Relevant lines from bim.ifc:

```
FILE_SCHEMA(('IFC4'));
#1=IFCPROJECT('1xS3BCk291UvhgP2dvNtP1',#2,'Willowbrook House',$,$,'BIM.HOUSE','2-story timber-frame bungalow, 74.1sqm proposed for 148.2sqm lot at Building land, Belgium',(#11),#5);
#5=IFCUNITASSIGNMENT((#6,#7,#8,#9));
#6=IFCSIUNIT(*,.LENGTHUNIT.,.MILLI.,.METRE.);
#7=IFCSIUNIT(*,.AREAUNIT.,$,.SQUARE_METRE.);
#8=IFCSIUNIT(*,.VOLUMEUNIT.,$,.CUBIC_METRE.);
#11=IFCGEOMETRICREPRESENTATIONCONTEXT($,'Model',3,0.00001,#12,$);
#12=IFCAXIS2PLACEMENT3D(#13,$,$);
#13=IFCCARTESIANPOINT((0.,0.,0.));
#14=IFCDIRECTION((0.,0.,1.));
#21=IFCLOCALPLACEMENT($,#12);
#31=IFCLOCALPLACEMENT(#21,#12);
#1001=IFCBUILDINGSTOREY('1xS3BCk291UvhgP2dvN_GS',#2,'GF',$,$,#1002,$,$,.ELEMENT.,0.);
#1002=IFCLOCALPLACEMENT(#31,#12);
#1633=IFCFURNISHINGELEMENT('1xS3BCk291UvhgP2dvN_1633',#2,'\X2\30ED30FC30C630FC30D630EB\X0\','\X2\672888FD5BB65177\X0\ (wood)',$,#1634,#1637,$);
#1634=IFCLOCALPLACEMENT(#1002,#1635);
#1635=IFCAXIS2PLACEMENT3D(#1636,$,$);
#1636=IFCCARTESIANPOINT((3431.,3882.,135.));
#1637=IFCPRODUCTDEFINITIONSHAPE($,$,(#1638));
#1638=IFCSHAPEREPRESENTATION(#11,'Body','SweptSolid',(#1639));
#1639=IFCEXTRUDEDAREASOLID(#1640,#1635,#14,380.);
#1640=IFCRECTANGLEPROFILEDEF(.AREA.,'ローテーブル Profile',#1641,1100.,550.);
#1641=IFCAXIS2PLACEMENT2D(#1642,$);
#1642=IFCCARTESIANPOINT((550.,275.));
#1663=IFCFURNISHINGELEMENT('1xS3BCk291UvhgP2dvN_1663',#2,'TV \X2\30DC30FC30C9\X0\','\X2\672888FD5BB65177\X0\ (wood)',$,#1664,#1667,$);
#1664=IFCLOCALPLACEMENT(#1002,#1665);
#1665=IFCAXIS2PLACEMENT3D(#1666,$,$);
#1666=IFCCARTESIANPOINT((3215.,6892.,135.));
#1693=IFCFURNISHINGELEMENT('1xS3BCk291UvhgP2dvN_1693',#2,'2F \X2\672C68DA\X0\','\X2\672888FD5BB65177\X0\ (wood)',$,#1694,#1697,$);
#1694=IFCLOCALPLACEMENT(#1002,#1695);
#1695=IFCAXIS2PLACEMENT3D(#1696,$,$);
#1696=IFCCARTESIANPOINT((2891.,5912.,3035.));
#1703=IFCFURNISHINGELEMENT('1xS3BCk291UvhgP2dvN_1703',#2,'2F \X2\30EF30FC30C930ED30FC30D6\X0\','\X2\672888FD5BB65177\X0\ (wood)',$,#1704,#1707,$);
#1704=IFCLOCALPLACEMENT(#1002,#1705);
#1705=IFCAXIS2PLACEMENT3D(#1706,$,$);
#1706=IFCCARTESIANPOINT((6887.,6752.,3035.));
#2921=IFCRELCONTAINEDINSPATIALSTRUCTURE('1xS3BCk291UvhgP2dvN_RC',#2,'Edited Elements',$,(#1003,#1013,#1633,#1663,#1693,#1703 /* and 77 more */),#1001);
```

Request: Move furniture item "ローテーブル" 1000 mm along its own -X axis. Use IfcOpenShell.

```python
import ifcopenshell
import ifcopenshell.api.geometry
import ifcopenshell.util.placement

model = ifcopenshell.open("bim.ifc")

item = model.by_id(1633)
matrix = ifcopenshell.util.placement.get_local_placement(item.ObjectPlacement)
matrix[:3, 3] -= matrix[:3, 0] * 1000.0
ifcopenshell.api.geometry.edit_object_placement(model, product=item, matrix=matrix, is_si=False)

print(ifcopenshell.util.placement.get_local_placement(item.ObjectPlacement).round(3) + 0.0)

model.write("bim_v2.ifc")
```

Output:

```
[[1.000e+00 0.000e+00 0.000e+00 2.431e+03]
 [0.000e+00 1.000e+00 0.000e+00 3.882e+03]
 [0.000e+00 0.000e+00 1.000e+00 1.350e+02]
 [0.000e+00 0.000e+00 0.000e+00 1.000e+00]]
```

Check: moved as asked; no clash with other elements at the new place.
